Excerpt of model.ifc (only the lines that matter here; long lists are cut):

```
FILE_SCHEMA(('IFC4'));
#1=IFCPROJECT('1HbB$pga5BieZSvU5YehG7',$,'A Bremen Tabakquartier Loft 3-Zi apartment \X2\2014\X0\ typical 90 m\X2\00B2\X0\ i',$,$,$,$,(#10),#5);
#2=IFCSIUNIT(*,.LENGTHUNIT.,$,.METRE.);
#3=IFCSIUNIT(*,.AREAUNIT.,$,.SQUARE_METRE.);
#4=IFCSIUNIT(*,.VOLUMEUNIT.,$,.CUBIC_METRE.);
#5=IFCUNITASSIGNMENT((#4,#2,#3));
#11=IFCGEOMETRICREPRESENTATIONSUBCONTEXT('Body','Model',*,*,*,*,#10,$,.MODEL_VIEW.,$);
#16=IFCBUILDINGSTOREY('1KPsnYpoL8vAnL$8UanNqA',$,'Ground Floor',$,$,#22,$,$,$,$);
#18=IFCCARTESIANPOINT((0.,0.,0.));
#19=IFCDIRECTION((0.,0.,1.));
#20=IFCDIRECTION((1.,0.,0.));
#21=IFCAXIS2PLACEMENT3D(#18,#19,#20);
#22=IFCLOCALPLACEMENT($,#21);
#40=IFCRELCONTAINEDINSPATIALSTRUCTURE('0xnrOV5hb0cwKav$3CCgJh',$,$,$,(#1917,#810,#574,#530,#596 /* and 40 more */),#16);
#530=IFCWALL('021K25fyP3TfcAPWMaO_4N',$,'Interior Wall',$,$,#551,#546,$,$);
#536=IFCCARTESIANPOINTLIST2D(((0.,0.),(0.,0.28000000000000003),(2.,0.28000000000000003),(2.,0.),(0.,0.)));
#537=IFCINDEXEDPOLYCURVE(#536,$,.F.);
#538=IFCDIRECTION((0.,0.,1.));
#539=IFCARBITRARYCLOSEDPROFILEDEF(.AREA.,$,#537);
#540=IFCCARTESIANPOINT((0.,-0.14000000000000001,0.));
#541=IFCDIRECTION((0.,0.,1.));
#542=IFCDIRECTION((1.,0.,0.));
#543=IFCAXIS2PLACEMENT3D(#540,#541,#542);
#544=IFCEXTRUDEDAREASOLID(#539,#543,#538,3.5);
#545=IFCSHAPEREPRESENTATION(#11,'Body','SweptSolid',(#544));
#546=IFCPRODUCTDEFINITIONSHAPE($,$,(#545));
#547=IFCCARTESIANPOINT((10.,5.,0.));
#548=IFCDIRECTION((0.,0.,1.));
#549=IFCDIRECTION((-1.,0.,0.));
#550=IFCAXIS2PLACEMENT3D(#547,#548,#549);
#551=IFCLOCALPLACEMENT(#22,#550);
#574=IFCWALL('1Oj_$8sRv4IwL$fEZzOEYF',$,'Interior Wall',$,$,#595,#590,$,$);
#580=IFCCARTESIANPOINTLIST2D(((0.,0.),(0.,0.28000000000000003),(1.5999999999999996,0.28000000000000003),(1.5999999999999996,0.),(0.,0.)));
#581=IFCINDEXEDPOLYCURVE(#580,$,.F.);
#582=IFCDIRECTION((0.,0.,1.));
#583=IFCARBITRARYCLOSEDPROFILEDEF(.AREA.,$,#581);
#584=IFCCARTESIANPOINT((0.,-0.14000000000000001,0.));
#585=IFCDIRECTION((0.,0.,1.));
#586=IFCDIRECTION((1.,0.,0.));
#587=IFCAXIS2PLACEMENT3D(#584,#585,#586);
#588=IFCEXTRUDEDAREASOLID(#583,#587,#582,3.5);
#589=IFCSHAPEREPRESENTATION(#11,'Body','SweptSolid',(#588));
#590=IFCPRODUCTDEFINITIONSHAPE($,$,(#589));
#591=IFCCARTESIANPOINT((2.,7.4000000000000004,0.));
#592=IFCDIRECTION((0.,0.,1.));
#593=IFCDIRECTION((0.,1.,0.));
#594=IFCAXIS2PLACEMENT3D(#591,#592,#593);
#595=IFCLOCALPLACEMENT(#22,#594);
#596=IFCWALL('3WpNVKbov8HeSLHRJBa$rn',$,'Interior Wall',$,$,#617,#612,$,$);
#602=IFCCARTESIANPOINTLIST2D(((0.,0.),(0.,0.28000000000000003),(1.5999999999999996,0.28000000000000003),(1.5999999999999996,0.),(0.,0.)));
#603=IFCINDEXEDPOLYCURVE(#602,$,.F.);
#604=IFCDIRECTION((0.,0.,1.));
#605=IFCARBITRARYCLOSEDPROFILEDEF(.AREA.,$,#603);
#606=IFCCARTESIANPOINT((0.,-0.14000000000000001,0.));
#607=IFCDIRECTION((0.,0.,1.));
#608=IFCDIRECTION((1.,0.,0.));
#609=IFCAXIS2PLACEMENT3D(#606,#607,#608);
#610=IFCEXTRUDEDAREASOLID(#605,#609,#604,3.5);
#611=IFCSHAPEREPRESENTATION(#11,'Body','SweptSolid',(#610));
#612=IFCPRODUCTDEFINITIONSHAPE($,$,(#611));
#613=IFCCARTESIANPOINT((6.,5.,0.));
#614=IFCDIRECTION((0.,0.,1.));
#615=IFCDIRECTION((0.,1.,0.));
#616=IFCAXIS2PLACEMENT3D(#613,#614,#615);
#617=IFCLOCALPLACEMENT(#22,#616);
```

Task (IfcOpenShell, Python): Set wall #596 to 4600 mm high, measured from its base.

```python
import ifcopenshell
import ifcopenshell.geom
import ifcopenshell.util.representation
import ifcopenshell.util.shape
import ifcopenshell.util.unit

model = ifcopenshell.open("model.ifc")
unit_scale = ifcopenshell.util.unit.calculate_unit_scale(model)
settings = ifcopenshell.geom.settings()


def volume(element):
    """Net volume in cubic metres, openings subtracted."""
    shape = ifcopenshell.geom.create_shape(settings, element)
    return ifcopenshell.util.shape.get_volume(shape.geometry)


wall = model.by_guid("3WpNVKbov8HeSLHRJBa$rn")
before = volume(wall)

body = ifcopenshell.util.representation.get_representation(wall, "Model", "Body")
solid = body.Items[0]
old_height = solid.Depth
solid.Depth = 4.6 / unit_scale
after = volume(wall)

print(f"height {old_height:g} -> {solid.Depth:g}, volume {before:.3f} -> {after:.3f} m3")

model.write("model_v2.ifc")
```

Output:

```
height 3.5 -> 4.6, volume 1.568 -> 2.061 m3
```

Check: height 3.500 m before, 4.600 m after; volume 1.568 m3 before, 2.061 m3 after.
